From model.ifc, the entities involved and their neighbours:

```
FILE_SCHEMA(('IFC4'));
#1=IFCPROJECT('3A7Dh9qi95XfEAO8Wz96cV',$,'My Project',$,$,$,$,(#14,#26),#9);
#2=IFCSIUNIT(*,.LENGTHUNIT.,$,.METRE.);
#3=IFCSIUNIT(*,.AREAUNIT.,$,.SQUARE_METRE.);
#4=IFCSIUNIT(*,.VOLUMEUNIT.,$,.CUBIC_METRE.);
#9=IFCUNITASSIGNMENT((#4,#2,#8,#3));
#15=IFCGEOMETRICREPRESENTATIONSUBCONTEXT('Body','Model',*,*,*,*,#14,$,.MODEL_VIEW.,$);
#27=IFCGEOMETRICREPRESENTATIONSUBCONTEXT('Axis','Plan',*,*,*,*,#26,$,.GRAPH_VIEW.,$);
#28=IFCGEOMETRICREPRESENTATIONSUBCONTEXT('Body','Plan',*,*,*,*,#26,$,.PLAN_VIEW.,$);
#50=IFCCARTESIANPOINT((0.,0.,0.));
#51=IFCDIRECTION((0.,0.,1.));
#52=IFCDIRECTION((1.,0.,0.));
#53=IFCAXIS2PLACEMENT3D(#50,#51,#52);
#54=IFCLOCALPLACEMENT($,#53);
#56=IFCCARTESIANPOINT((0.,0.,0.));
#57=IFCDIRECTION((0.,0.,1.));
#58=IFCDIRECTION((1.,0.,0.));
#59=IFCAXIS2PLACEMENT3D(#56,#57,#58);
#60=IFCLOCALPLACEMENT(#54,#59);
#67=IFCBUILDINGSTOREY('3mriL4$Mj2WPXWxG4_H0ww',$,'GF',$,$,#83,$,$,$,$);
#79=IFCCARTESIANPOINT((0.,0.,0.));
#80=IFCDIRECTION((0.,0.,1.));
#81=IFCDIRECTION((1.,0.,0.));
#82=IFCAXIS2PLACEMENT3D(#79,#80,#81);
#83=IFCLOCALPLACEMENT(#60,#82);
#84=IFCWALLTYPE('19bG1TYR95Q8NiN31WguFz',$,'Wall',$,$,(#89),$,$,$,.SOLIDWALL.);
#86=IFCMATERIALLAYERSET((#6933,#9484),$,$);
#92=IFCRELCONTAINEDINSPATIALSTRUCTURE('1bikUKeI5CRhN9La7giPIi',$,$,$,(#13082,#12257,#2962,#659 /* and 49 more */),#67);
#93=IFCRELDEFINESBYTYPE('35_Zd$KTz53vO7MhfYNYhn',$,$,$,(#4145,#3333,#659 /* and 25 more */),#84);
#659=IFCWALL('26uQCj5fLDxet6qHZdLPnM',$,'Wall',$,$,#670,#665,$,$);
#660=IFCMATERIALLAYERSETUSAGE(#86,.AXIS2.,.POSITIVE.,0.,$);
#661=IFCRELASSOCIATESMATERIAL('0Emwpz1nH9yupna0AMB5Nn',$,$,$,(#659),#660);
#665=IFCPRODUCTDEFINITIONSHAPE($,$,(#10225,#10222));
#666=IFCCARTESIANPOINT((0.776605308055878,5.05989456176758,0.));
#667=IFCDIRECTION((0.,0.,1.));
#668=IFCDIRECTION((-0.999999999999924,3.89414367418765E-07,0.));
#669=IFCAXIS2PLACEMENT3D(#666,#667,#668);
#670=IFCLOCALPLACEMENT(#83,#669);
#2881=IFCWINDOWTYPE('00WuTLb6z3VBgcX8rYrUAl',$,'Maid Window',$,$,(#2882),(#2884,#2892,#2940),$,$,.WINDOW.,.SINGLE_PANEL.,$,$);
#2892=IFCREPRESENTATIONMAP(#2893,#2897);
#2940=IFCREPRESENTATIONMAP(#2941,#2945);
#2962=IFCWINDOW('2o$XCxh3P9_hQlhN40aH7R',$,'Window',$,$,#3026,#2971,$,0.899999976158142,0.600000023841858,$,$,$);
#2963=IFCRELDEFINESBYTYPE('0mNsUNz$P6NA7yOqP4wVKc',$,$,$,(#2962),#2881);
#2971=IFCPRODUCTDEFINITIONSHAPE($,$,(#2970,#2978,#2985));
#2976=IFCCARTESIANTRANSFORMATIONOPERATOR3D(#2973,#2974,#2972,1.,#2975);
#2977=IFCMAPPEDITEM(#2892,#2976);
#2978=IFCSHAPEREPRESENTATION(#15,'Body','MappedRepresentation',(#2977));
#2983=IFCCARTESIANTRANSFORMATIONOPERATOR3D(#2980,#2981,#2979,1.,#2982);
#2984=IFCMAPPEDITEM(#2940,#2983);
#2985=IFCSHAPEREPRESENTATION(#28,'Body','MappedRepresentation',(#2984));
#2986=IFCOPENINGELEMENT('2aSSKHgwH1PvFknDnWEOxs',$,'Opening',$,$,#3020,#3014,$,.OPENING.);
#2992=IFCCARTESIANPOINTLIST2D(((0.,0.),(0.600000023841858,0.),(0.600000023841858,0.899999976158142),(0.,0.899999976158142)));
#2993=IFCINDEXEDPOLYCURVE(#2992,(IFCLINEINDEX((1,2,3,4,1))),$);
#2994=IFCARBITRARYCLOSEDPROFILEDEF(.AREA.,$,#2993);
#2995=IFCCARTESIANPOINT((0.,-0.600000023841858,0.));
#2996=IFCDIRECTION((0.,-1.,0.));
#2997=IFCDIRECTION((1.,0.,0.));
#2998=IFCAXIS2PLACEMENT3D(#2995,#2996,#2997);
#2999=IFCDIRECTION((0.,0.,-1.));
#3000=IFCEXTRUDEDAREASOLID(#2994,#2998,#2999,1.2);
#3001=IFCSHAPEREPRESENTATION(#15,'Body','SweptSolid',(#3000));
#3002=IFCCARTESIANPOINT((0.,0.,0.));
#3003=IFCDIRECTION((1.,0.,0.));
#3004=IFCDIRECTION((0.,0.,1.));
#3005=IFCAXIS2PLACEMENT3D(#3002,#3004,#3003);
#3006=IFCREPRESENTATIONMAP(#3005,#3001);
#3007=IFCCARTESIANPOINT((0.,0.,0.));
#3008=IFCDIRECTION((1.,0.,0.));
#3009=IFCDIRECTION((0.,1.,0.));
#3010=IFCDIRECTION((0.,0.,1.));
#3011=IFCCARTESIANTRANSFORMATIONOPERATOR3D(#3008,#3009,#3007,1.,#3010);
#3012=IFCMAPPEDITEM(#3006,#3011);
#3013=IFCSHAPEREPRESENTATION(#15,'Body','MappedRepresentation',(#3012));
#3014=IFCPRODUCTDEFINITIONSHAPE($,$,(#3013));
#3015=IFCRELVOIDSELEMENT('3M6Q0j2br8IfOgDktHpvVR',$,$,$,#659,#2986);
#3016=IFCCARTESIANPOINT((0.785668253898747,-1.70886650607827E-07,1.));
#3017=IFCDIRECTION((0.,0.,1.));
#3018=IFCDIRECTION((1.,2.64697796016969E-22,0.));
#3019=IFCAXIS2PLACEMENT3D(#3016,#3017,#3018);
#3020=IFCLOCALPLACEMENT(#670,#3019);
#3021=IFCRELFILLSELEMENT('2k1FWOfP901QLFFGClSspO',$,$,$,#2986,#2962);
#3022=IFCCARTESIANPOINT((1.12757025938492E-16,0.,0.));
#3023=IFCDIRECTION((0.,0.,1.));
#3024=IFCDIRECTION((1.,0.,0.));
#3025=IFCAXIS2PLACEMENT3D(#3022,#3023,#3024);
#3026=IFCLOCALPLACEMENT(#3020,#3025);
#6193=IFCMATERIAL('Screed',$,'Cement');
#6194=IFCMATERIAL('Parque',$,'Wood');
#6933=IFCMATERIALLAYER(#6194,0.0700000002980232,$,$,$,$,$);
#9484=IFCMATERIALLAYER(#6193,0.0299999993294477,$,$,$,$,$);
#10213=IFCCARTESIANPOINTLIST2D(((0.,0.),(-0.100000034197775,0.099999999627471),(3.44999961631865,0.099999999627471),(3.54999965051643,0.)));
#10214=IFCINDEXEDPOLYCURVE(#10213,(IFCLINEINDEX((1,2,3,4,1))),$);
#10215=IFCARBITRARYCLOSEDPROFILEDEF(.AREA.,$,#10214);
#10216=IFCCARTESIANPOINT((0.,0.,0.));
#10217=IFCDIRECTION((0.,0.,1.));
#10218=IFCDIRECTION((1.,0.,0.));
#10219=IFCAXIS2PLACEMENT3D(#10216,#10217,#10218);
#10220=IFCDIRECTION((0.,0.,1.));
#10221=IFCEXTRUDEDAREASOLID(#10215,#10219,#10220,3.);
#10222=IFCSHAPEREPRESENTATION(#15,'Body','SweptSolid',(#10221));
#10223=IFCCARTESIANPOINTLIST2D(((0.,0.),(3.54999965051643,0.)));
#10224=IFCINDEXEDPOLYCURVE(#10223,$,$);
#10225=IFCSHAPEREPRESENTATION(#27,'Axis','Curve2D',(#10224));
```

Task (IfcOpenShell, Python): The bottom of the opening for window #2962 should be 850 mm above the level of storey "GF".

```python
import numpy as np
import ifcopenshell
import ifcopenshell.api.geometry
import ifcopenshell.geom
import ifcopenshell.util.element
import ifcopenshell.util.placement
import ifcopenshell.util.shape
import ifcopenshell.util.unit

model = ifcopenshell.open("model.ifc")
unit_scale = ifcopenshell.util.unit.calculate_unit_scale(model)

window = model.by_id(2962)
opening = window.FillsVoids[0].RelatingOpeningElement
storey = ifcopenshell.util.element.get_container(window, ifc_class="IfcBuildingStorey")
level = ifcopenshell.util.placement.get_local_placement(storey.ObjectPlacement)[2, 3]

# The opening's origin need not be at the sill, so measure its lowest point.
shape = ifcopenshell.geom.create_shape(ifcopenshell.geom.settings(), opening)
bottom = ifcopenshell.util.shape.get_shape_bottom_elevation(shape, shape.geometry) / unit_scale
dz = level + 0.85 / unit_scale - bottom

shift = np.array([0.0, 0.0, dz])
# The window is placed relative to its opening, so it follows when the opening moves.
matrix = ifcopenshell.util.placement.get_local_placement(opening.ObjectPlacement)
matrix[:3, 3] += shift
ifcopenshell.api.geometry.edit_object_placement(
    model, product=opening, matrix=matrix, is_si=False, should_transform_children=True
)

print(f"moved by {dz * unit_scale:+.3f} m")

model.write("model-out.ifc")
```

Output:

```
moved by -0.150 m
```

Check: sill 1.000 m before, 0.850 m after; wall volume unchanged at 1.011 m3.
